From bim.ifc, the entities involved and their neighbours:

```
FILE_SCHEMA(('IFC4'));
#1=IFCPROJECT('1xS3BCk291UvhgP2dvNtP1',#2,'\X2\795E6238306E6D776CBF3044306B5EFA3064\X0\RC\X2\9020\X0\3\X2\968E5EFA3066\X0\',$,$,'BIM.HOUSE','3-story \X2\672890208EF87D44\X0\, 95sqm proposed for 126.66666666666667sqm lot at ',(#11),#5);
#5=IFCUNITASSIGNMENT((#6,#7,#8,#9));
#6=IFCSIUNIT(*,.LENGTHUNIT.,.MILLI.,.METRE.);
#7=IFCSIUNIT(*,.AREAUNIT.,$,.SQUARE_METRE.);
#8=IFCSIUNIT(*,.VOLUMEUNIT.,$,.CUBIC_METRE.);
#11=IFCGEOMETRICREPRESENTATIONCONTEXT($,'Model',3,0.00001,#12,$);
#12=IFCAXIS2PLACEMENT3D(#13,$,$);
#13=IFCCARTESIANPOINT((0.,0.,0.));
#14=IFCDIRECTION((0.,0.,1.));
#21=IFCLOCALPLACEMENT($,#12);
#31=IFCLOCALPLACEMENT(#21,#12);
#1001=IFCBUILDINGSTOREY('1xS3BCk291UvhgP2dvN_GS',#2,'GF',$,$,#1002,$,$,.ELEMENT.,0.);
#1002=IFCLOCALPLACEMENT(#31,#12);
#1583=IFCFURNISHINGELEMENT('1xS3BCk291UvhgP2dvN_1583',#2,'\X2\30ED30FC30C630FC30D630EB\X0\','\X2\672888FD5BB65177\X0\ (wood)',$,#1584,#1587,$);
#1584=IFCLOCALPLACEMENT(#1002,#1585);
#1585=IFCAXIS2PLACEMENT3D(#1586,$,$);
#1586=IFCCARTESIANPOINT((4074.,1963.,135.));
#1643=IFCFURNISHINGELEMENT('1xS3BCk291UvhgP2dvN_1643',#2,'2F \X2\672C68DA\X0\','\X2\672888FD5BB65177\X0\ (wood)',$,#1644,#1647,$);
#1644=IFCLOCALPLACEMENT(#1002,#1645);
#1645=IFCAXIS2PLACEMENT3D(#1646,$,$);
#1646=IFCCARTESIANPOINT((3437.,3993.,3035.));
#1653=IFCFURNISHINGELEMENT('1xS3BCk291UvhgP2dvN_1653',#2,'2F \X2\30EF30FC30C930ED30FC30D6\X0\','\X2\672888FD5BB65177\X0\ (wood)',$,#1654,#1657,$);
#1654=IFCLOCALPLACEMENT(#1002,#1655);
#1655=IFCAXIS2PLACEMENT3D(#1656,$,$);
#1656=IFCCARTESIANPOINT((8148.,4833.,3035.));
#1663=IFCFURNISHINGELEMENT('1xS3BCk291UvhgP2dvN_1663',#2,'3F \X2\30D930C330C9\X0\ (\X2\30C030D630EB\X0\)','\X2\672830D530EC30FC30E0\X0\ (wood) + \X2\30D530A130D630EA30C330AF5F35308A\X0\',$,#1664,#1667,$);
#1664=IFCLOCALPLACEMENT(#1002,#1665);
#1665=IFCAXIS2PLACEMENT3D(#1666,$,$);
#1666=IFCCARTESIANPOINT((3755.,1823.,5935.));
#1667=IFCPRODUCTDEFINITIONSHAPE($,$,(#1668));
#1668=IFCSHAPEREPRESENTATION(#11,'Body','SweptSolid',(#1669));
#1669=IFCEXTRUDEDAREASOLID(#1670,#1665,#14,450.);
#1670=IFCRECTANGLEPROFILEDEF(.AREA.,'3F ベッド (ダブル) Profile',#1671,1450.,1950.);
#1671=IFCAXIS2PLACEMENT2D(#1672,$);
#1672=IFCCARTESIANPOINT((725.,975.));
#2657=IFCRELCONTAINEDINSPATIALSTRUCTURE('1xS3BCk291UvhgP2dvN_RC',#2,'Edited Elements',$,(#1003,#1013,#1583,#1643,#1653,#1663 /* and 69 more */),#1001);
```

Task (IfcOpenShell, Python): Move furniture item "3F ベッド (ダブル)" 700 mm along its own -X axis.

```python
import ifcopenshell
import ifcopenshell.api.geometry
import ifcopenshell.util.placement

model = ifcopenshell.open("bim.ifc")

item = model.by_guid("1xS3BCk291UvhgP2dvN_1663")
matrix = ifcopenshell.util.placement.get_local_placement(item.ObjectPlacement)
matrix[:3, 3] -= matrix[:3, 0] * 700.0
ifcopenshell.api.geometry.edit_object_placement(model, product=item, matrix=matrix, is_si=False)

print(ifcopenshell.util.placement.get_local_placement(item.ObjectPlacement).round(3) + 0.0)

model.write("bim_updated.ifc")
```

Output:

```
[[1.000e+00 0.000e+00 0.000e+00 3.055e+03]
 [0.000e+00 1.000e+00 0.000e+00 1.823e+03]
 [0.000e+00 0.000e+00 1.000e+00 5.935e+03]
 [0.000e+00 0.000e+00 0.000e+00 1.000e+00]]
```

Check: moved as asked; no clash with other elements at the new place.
